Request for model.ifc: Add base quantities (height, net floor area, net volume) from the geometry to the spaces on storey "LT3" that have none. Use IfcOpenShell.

First a look at what the model holds.

```python
import ifcopenshell
import ifcopenshell.util.element
import ifcopenshell.util.unit

model = ifcopenshell.open("model.ifc")
print(model.schema)
for unit_type in ("LENGTHUNIT", "AREAUNIT", "VOLUMEUNIT"):
    print(unit_type, ifcopenshell.util.unit.calculate_unit_scale(model, unit_type))
storey = next(s for s in model.by_type("IfcBuildingStorey") if s.Name == "LT3")
spaces = [e for e in ifcopenshell.util.element.get_decomposition(storey) if e.is_a("IfcSpace")]
for e in sorted(spaces, key=lambda e: e.id()):
    print(e.id(), e.is_a(), e.Name, list(ifcopenshell.util.element.get_psets(e, qtos_only=True)), sep=" | ")
```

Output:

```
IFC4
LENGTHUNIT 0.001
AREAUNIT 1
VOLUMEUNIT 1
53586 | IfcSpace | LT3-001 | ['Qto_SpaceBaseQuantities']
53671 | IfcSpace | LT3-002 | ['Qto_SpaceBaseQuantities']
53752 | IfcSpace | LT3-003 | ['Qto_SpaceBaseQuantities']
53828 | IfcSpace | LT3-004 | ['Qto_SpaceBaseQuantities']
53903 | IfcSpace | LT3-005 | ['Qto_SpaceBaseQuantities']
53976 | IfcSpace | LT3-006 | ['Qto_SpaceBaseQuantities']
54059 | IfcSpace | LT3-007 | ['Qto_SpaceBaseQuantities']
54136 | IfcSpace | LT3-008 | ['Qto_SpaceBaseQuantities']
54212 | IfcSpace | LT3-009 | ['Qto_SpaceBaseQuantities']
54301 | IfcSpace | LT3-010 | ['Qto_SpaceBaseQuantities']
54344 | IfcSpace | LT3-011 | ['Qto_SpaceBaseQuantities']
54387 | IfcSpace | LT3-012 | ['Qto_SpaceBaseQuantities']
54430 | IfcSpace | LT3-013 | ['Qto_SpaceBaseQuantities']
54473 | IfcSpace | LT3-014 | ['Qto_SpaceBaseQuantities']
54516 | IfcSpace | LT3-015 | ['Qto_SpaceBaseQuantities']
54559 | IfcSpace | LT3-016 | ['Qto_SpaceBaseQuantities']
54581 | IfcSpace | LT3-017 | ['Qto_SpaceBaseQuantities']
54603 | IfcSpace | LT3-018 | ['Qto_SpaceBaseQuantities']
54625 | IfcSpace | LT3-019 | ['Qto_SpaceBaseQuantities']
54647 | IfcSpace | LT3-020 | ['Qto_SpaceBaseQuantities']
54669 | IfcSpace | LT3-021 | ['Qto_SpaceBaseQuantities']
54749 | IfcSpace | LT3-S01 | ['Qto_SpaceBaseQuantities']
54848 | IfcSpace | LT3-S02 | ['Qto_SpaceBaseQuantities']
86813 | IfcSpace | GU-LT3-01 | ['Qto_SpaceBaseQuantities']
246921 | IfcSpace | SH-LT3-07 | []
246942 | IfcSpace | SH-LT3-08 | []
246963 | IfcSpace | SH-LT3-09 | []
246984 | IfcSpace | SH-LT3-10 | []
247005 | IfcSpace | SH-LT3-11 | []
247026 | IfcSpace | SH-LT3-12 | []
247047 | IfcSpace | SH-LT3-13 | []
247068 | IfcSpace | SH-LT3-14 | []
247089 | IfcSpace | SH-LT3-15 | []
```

```python
import ifcopenshell
import ifcopenshell.api.pset
import ifcopenshell.geom
import ifcopenshell.util.element
import ifcopenshell.util.shape
import ifcopenshell.util.unit

model = ifcopenshell.open("model.ifc")
unit_scale = ifcopenshell.util.unit.calculate_unit_scale(model)
area_scale = ifcopenshell.util.unit.calculate_unit_scale(model, "AREAUNIT")
volume_scale = ifcopenshell.util.unit.calculate_unit_scale(model, "VOLUMEUNIT")
settings = ifcopenshell.geom.settings()

storey = next(s for s in model.by_type("IfcBuildingStorey") if s.Name == "LT3")
spaces = [e for e in ifcopenshell.util.element.get_decomposition(storey) if e.is_a("IfcSpace")]

for e in sorted(spaces, key=lambda e: e.id()):
    if ifcopenshell.util.element.get_psets(e, qtos_only=True, should_inherit=False):
        continue
    # Geometry comes back in metres, in the element's own axes.
    shape = ifcopenshell.geom.create_shape(settings, e)
    values = {
        "Height": ifcopenshell.util.shape.get_z(shape.geometry) / unit_scale,
        "NetFloorArea": ifcopenshell.util.shape.get_footprint_area(shape.geometry) / area_scale,
        "NetVolume": ifcopenshell.util.shape.get_volume(shape.geometry) / volume_scale,
    }
    qto = ifcopenshell.api.pset.add_qto(model, product=e, name="Qto_SpaceBaseQuantities")
    ifcopenshell.api.pset.edit_qto(model, qto=qto, properties=values)
    print(e.id(), {k: round(v, 3) for k, v in values.items()})

model.write("model_rev.ifc")
```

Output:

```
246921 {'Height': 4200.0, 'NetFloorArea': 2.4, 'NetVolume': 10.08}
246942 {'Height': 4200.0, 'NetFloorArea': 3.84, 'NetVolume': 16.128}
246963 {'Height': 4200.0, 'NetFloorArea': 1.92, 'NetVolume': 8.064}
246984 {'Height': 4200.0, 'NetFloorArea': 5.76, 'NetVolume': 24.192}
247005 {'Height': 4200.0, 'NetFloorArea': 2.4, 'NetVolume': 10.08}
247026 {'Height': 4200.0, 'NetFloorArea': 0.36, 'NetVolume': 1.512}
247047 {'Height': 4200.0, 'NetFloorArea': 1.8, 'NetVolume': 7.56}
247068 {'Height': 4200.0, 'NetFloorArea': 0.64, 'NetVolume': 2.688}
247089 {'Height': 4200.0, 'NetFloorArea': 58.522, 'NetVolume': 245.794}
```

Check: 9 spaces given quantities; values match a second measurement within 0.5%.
